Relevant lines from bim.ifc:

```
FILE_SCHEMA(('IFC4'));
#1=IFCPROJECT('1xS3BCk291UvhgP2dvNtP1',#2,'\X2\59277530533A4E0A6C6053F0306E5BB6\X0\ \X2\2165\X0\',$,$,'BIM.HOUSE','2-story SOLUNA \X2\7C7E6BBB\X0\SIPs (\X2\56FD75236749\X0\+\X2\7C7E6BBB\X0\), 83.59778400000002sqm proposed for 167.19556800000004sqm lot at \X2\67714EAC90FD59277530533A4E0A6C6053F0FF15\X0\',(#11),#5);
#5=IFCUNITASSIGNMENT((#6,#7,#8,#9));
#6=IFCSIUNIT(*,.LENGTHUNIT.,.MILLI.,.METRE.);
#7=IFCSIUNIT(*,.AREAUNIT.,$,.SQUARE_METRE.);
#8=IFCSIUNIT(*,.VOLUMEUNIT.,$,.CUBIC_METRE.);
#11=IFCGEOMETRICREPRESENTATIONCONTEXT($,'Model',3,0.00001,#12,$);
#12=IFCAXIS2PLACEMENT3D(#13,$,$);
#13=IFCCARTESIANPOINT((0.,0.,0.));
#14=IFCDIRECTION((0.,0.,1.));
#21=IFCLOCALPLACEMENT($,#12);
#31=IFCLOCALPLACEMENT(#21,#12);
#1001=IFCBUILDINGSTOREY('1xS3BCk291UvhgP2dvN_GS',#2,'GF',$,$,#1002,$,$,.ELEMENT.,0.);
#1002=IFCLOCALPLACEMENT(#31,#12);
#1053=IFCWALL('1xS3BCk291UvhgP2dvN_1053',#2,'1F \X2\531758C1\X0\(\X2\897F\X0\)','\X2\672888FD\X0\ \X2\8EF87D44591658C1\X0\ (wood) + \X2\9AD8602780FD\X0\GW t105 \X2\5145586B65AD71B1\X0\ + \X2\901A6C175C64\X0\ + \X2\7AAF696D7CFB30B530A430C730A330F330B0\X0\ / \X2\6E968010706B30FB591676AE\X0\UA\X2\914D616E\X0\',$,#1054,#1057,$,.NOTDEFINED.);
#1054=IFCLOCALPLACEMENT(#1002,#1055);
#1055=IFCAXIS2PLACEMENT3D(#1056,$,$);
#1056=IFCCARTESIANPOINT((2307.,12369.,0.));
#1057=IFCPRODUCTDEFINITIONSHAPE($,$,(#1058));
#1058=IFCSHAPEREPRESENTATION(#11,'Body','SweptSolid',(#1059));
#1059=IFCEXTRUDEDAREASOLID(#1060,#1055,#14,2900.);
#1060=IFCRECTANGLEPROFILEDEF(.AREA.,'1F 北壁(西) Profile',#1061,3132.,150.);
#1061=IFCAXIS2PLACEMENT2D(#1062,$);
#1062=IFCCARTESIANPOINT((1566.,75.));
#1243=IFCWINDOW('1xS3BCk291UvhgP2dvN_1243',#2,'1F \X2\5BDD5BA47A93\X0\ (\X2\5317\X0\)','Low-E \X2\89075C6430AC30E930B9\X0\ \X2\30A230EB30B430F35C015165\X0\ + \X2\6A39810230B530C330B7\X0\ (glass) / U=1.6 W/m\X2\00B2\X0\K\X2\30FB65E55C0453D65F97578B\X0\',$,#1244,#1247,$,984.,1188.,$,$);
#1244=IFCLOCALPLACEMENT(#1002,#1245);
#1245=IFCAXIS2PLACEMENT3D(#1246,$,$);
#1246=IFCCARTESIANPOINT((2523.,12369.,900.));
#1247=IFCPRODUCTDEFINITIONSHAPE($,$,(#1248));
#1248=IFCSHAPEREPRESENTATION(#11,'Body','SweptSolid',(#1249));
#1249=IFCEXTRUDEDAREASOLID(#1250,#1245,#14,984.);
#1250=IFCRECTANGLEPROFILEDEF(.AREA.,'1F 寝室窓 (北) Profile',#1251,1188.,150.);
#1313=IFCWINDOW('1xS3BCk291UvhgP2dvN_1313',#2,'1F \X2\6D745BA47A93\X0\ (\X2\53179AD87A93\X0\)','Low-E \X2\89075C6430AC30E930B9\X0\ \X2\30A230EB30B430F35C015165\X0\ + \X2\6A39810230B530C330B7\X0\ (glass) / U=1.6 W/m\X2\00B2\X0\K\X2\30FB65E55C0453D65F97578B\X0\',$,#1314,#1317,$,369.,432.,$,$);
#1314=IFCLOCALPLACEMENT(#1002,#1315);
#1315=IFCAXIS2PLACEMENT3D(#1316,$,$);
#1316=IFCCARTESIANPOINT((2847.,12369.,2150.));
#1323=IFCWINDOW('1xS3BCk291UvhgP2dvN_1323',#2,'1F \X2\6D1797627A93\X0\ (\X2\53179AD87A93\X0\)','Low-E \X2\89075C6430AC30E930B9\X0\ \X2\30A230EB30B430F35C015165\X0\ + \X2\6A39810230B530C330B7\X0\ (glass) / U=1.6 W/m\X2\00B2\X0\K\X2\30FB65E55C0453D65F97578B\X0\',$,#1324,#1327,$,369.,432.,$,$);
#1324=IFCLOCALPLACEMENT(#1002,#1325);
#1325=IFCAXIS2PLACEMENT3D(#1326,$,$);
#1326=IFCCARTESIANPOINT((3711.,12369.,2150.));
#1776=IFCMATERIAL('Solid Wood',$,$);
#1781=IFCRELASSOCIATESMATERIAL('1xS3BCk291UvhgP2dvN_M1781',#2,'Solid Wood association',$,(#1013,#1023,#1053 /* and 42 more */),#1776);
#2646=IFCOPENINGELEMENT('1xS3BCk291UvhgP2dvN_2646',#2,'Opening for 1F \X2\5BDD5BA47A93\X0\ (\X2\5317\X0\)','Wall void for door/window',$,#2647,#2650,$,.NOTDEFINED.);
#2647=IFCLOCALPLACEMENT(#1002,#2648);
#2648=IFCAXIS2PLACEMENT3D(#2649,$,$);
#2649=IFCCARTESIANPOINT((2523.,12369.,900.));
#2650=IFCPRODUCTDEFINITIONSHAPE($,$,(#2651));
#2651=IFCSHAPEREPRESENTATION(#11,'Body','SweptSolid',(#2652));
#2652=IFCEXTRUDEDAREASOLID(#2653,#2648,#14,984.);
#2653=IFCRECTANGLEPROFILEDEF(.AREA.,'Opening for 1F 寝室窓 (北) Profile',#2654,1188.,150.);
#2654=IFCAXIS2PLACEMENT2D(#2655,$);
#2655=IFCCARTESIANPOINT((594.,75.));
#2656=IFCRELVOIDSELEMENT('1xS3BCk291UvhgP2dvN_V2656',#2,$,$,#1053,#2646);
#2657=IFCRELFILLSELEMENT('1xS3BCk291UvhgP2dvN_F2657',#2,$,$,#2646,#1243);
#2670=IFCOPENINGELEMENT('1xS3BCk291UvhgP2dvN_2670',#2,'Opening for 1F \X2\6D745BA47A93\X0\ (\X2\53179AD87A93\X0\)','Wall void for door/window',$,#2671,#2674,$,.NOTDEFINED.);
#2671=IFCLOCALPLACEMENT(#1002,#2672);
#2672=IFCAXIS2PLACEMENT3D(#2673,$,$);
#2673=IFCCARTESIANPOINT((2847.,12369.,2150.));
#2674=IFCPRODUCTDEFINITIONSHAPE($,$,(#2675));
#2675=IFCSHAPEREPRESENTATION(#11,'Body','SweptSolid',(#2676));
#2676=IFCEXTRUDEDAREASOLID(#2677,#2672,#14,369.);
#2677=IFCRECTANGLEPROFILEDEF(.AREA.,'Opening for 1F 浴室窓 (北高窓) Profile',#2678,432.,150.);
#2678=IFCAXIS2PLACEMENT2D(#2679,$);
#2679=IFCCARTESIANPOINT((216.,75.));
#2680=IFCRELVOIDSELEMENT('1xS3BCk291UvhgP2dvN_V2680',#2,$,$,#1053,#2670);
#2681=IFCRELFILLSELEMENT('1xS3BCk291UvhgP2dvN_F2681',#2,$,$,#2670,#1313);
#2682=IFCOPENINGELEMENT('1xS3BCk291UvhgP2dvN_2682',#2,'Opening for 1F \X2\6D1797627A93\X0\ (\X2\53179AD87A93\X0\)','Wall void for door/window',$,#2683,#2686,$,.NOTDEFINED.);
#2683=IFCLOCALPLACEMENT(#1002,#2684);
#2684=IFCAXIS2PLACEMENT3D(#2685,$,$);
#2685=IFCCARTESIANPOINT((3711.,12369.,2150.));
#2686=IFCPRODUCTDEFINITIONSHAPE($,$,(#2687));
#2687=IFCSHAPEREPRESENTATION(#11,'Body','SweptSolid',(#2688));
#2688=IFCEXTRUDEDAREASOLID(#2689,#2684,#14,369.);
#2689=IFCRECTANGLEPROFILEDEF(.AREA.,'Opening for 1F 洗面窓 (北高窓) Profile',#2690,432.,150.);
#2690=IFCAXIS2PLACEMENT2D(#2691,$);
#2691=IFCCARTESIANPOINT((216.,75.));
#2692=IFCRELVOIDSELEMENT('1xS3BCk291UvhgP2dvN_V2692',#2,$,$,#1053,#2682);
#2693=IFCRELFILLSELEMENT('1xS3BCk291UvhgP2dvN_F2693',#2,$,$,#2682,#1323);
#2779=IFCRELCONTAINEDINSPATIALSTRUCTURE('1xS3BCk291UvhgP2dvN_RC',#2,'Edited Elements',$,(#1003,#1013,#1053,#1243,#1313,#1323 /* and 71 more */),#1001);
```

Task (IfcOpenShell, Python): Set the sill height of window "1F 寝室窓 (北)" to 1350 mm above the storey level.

```python
import numpy as np
import ifcopenshell
import ifcopenshell.api.geometry
import ifcopenshell.geom
import ifcopenshell.util.element
import ifcopenshell.util.placement
import ifcopenshell.util.shape
import ifcopenshell.util.unit

model = ifcopenshell.open("bim.ifc")
unit_scale = ifcopenshell.util.unit.calculate_unit_scale(model)

window = model.by_guid("1xS3BCk291UvhgP2dvN_1243")
opening = window.FillsVoids[0].RelatingOpeningElement
storey = ifcopenshell.util.element.get_container(window, ifc_class="IfcBuildingStorey")
level = ifcopenshell.util.placement.get_local_placement(storey.ObjectPlacement)[2, 3]

# The opening's origin need not be at the sill, so measure its lowest point.
shape = ifcopenshell.geom.create_shape(ifcopenshell.geom.settings(), opening)
bottom = ifcopenshell.util.shape.get_shape_bottom_elevation(shape, shape.geometry) / unit_scale
dz = level + 1350.0 - bottom

shift = np.array([0.0, 0.0, dz])
# The window is not placed relative to its opening, so move both.
for product in (opening, window):
    matrix = ifcopenshell.util.placement.get_local_placement(product.ObjectPlacement)
    matrix[:3, 3] += shift
    ifcopenshell.api.geometry.edit_object_placement(model, product=product, matrix=matrix, is_si=False)

print(f"moved by {dz * unit_scale:+.3f} m")

model.write("bim-out.ifc")
```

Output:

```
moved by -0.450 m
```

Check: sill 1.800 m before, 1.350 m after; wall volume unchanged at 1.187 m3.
